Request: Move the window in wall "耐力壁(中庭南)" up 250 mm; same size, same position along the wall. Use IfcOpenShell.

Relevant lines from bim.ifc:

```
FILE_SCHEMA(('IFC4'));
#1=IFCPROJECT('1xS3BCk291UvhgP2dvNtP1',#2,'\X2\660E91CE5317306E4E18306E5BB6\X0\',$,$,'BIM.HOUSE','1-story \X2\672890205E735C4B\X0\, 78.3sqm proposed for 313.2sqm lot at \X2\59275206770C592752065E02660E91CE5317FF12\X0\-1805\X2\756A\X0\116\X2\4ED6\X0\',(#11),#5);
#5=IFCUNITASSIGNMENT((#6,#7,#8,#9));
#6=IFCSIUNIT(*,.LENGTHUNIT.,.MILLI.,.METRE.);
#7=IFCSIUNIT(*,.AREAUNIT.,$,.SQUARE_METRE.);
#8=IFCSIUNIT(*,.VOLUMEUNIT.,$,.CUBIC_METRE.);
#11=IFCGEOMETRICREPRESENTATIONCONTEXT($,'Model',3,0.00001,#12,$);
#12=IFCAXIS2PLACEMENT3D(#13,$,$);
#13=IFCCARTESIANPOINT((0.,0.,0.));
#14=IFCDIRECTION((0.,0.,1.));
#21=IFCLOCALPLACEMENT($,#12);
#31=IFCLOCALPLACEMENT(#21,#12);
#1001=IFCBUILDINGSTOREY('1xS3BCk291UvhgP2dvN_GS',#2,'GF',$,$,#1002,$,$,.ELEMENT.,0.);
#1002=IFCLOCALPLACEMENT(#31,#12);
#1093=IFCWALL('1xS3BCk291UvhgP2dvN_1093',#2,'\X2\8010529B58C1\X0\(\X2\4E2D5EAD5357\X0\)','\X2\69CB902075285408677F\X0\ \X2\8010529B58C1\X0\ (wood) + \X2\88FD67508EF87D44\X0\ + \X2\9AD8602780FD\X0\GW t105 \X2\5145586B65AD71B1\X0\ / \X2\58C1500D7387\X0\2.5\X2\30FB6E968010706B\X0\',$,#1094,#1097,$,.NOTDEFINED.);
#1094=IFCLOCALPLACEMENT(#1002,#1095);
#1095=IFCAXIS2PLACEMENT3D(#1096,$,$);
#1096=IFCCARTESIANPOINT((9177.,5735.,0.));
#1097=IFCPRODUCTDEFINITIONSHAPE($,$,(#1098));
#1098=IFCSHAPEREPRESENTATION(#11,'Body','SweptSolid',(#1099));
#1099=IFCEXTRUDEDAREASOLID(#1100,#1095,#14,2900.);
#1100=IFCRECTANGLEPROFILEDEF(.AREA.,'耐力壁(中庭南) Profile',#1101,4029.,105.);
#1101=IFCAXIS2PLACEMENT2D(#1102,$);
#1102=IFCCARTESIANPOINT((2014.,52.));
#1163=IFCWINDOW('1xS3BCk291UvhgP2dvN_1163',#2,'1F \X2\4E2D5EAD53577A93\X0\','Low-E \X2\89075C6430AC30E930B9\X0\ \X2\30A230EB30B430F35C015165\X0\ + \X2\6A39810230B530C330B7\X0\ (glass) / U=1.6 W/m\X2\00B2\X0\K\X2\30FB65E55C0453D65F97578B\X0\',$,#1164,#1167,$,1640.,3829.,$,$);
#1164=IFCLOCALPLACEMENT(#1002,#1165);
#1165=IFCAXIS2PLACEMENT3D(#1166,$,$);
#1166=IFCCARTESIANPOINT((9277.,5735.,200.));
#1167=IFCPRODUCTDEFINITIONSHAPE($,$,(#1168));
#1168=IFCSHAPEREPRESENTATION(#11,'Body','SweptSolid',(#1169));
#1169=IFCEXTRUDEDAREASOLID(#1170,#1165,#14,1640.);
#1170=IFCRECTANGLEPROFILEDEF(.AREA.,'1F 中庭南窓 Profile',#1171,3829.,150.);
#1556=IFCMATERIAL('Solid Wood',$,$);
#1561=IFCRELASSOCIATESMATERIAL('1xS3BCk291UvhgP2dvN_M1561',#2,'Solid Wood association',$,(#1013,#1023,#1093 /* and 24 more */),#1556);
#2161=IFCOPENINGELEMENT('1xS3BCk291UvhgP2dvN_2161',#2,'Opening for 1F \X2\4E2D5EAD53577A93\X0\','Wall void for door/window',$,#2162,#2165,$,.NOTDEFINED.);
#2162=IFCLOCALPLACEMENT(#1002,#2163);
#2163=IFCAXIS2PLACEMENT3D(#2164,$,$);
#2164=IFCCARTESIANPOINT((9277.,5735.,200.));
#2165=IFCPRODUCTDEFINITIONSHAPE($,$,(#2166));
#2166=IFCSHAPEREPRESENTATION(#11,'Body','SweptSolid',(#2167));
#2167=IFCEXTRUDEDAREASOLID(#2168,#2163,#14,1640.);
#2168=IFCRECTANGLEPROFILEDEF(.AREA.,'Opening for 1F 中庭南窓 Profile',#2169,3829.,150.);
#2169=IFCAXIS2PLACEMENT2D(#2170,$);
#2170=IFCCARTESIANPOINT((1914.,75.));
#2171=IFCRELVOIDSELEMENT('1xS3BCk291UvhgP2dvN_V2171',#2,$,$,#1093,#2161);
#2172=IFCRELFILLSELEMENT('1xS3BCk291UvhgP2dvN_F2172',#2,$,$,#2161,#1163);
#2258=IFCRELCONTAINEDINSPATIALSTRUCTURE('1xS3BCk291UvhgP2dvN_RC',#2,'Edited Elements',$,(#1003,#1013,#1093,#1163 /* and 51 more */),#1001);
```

```python
import numpy as np
import ifcopenshell
import ifcopenshell.api.geometry
import ifcopenshell.util.placement
import ifcopenshell.util.unit

model = ifcopenshell.open("bim.ifc")
unit_scale = ifcopenshell.util.unit.calculate_unit_scale(model)

window = model.by_guid("1xS3BCk291UvhgP2dvN_1163")
opening = window.FillsVoids[0].RelatingOpeningElement
dz = 250.0

shift = np.array([0.0, 0.0, dz])
# The window is not placed relative to its opening, so move both.
for product in (opening, window):
    matrix = ifcopenshell.util.placement.get_local_placement(product.ObjectPlacement)
    matrix[:3, 3] += shift
    ifcopenshell.api.geometry.edit_object_placement(model, product=product, matrix=matrix, is_si=False)

print(f"moved by {dz * unit_scale:+.3f} m")

model.write("bim_rev.ifc")
```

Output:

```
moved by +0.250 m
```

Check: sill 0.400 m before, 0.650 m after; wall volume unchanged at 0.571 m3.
